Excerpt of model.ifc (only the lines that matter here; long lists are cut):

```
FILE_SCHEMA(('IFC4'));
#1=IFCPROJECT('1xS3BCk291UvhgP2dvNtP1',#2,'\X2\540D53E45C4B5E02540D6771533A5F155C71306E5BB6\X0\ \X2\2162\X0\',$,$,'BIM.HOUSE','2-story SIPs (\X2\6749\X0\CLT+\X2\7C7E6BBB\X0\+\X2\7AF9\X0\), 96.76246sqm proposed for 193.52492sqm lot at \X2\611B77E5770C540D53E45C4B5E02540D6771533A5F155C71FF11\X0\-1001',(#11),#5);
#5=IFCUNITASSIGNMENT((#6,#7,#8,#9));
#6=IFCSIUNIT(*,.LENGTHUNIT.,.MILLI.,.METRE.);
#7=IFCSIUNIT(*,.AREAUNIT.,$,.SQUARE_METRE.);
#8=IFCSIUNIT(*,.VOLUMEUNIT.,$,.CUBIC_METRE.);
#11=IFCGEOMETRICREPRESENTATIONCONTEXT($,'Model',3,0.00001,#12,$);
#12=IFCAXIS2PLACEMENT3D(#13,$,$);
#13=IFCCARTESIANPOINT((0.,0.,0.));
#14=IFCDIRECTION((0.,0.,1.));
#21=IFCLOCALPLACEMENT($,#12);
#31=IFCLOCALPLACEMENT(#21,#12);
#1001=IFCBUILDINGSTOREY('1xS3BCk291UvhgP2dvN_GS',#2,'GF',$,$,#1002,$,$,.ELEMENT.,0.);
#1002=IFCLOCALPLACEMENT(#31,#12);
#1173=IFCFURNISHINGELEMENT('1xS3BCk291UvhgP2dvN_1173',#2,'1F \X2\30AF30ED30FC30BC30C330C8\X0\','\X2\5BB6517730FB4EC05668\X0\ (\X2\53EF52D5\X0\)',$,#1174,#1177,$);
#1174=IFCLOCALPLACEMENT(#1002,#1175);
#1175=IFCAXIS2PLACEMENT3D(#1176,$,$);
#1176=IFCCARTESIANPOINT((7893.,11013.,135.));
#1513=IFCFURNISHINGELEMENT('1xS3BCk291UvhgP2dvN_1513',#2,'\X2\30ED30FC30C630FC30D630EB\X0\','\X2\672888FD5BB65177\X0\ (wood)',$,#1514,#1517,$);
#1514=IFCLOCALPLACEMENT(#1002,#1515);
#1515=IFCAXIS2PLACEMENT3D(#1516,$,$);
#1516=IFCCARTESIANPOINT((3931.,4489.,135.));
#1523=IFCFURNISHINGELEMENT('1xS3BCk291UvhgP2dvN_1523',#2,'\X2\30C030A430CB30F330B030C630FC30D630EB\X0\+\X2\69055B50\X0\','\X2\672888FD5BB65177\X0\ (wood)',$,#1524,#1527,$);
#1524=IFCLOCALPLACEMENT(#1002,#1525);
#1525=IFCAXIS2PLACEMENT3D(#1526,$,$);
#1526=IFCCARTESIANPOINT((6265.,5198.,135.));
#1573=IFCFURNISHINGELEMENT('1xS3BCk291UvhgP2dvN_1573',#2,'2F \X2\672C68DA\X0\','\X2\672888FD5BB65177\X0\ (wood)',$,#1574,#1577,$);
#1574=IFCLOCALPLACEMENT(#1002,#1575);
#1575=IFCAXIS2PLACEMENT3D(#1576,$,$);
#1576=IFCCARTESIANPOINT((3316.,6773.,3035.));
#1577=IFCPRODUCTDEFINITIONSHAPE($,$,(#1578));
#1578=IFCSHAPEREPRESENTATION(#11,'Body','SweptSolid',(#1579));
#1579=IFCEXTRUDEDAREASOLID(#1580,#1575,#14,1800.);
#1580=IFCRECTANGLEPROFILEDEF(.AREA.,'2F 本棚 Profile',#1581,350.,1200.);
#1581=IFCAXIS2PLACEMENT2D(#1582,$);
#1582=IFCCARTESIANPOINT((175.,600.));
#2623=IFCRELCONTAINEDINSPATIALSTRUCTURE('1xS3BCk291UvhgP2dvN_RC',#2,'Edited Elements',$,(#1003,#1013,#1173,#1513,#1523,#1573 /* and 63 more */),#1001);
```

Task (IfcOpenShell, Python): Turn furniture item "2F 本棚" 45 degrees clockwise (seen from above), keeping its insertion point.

```python
import ifcopenshell
import ifcopenshell.api.geometry
import ifcopenshell.util.placement

model = ifcopenshell.open("model.ifc")

item = model.by_guid("1xS3BCk291UvhgP2dvN_1573")
matrix = ifcopenshell.util.placement.get_local_placement(item.ObjectPlacement)
matrix = matrix @ ifcopenshell.util.placement.rotation(-45, "Z")
ifcopenshell.api.geometry.edit_object_placement(model, product=item, matrix=matrix, is_si=False)

print(ifcopenshell.util.placement.get_local_placement(item.ObjectPlacement).round(3) + 0.0)

model.write("model_rev.ifc")
```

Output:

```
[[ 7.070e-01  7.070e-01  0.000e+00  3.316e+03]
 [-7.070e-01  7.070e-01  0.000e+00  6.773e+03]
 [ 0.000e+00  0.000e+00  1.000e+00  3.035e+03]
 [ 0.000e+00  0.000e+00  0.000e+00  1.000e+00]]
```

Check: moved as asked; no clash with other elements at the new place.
